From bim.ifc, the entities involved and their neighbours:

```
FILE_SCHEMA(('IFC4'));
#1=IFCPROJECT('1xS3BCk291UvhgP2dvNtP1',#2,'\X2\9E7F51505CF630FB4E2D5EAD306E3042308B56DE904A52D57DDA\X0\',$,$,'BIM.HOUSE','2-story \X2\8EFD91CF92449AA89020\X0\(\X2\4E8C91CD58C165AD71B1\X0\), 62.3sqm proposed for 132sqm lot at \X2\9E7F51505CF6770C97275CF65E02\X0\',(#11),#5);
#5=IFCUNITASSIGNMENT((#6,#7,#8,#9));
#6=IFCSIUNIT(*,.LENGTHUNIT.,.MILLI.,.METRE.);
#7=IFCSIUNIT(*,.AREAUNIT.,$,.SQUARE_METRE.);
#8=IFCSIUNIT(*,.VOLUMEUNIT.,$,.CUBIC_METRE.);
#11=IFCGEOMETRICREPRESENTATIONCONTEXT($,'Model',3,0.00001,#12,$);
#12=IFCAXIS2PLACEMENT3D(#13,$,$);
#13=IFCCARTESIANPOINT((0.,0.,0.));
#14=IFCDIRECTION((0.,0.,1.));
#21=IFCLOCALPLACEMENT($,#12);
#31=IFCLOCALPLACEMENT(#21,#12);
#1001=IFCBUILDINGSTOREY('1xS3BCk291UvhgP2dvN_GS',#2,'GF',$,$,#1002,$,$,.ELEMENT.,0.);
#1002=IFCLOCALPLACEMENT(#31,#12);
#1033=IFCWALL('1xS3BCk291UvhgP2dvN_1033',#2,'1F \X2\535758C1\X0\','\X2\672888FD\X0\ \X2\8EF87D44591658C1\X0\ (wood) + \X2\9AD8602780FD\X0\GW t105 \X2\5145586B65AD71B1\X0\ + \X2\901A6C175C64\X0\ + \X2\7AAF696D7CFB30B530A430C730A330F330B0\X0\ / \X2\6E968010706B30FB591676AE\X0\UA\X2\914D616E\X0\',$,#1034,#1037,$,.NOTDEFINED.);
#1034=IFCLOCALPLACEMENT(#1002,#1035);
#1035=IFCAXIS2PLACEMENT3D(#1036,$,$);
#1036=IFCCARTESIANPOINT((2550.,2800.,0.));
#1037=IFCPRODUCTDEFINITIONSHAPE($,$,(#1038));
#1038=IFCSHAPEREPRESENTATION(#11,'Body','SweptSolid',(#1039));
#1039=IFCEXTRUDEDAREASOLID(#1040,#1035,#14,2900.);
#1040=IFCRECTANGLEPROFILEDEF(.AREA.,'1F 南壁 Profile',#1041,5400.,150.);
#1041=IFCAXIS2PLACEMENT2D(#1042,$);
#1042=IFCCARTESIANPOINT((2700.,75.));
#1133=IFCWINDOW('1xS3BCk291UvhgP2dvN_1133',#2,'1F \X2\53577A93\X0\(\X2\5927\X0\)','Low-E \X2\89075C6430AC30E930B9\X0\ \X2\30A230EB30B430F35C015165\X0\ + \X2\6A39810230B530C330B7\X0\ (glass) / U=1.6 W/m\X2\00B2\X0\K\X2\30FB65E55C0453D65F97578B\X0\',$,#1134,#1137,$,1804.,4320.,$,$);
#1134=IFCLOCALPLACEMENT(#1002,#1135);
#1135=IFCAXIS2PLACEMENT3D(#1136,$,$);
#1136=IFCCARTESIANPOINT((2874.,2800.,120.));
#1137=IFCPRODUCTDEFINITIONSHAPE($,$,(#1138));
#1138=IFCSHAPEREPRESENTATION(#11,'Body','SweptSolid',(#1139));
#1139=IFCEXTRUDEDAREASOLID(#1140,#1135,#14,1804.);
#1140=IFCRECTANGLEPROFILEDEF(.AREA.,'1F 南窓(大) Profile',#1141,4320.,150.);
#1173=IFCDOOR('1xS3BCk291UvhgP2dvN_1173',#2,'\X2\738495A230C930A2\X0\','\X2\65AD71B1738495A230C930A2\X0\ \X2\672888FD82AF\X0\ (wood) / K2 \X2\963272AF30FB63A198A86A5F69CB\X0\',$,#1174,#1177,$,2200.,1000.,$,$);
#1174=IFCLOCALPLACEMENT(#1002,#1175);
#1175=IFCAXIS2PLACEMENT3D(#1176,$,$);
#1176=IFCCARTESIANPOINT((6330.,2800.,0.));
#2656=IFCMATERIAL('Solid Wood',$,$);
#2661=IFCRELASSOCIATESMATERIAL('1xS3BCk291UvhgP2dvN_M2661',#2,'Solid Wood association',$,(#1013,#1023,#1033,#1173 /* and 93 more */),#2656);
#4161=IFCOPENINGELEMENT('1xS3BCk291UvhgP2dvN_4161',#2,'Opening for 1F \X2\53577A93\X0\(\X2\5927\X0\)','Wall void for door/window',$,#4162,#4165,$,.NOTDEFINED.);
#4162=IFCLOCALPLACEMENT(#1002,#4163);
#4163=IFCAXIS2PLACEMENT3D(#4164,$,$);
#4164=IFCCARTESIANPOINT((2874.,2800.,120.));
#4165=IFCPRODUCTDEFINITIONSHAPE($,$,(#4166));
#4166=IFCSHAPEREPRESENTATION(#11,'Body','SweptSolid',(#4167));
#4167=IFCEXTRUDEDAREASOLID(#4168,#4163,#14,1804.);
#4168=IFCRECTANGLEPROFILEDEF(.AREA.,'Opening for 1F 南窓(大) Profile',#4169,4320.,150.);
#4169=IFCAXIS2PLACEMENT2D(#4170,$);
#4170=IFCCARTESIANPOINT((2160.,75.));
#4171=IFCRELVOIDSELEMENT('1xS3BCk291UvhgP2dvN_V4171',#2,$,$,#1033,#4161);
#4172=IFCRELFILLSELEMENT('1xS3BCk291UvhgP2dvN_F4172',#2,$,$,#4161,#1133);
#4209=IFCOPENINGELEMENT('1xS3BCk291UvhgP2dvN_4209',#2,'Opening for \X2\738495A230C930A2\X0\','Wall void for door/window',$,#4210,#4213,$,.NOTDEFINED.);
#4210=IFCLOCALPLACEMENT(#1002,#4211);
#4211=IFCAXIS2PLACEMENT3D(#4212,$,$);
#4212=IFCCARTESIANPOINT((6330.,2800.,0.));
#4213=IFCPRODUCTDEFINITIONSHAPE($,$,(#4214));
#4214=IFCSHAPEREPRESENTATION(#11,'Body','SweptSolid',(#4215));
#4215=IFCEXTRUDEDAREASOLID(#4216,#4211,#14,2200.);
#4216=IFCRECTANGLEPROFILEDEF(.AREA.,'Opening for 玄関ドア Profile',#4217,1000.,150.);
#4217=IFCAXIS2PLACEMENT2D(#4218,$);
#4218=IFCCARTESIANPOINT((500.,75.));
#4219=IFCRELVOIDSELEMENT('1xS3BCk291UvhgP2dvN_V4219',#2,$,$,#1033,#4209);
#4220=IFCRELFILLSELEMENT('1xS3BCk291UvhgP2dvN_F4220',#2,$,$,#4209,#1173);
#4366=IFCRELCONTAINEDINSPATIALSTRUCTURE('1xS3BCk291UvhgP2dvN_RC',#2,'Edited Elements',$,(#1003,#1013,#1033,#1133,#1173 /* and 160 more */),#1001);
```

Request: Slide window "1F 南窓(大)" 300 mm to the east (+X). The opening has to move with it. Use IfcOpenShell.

```python
import ifcopenshell
import ifcopenshell.api.geometry
import ifcopenshell.util.placement
import ifcopenshell.util.unit

model = ifcopenshell.open("bim.ifc")
unit_scale = ifcopenshell.util.unit.calculate_unit_scale(model)

window = model.by_guid("1xS3BCk291UvhgP2dvN_1133")
opening = window.FillsVoids[0].RelatingOpeningElement
wall = opening.VoidsElements[0].RelatingBuildingElement

wall_matrix = ifcopenshell.util.placement.get_local_placement(wall.ObjectPlacement)
shift = wall_matrix[:3, 0] * 0.3 / unit_scale
before = ifcopenshell.util.placement.get_local_placement(window.ObjectPlacement)[:3, 3].copy()

# The window is not placed relative to its opening, so move both.
for product in (opening, window):
    matrix = ifcopenshell.util.placement.get_local_placement(product.ObjectPlacement)
    matrix[:3, 3] += shift
    ifcopenshell.api.geometry.edit_object_placement(model, product=product, matrix=matrix, is_si=False)

after = ifcopenshell.util.placement.get_local_placement(window.ObjectPlacement)[:3, 3]
print("window moved by", (after - before).round(3) + 0.0)

model.write("bim_rev.ifc")
```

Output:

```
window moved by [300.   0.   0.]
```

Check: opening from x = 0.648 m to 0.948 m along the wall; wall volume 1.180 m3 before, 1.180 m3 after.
